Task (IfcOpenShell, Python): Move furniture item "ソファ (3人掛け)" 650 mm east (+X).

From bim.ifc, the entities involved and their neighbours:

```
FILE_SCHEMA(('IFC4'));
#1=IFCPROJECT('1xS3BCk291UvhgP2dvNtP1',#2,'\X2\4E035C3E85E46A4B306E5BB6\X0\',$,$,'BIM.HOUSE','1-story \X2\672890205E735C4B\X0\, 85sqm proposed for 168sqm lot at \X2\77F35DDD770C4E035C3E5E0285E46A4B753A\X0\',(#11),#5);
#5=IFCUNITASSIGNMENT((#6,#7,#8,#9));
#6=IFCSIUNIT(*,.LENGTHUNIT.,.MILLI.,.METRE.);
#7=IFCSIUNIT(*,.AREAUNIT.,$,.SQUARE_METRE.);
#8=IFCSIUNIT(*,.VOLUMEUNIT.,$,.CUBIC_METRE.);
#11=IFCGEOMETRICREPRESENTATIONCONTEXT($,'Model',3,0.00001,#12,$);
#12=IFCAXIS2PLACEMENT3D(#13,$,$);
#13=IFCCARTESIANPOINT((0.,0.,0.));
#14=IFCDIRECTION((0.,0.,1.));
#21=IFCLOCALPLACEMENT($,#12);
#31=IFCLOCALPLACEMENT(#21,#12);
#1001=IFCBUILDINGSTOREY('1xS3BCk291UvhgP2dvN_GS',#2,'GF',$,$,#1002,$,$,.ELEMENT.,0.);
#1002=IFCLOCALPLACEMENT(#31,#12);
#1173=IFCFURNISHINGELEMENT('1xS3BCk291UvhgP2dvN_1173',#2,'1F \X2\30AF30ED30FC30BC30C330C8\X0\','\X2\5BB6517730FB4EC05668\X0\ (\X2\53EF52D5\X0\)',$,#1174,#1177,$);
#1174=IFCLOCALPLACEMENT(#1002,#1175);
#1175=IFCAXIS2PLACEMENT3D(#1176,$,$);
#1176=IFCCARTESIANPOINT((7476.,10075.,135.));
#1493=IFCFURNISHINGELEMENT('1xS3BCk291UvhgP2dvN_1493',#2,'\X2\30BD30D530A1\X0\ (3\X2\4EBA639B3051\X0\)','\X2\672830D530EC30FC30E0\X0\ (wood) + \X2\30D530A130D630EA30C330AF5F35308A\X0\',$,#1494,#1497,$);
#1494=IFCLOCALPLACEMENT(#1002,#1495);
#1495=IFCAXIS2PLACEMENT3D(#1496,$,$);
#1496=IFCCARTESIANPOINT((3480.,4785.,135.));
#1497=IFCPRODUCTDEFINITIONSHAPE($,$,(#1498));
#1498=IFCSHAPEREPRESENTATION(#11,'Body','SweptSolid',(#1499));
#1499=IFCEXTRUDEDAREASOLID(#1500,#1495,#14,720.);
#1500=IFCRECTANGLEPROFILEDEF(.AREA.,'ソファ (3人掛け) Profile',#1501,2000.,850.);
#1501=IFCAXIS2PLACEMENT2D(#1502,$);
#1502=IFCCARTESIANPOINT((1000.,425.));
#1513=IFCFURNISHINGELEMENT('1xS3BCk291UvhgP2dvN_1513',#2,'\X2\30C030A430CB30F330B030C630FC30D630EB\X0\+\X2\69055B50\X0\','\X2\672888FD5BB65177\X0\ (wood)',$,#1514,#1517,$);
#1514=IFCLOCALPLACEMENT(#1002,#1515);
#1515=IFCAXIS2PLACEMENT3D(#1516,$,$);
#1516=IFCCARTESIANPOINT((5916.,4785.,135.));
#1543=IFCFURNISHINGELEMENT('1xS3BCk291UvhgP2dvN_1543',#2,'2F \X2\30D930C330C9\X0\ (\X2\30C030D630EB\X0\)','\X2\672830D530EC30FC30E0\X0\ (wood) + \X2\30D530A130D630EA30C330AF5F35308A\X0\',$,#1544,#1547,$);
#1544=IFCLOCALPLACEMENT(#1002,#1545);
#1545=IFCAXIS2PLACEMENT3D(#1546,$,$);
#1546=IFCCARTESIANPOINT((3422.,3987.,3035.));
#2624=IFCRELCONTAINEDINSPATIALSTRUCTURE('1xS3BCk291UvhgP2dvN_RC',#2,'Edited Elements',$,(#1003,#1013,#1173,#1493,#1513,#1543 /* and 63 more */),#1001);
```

```python
import ifcopenshell
import ifcopenshell.api.geometry
import ifcopenshell.util.placement
import ifcopenshell.util.unit

model = ifcopenshell.open("bim.ifc")
unit_scale = ifcopenshell.util.unit.calculate_unit_scale(model)

item = model.by_guid("1xS3BCk291UvhgP2dvN_1493")
matrix = ifcopenshell.util.placement.get_local_placement(item.ObjectPlacement)
matrix[0, 3] += 0.65 / unit_scale
ifcopenshell.api.geometry.edit_object_placement(model, product=item, matrix=matrix, is_si=False)

print(ifcopenshell.util.placement.get_local_placement(item.ObjectPlacement).round(3) + 0.0)

model.write("bim_updated.ifc")
```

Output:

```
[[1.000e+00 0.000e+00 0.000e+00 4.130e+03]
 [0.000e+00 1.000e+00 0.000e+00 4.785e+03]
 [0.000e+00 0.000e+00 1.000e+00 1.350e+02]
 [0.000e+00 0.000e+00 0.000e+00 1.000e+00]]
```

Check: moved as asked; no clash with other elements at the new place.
